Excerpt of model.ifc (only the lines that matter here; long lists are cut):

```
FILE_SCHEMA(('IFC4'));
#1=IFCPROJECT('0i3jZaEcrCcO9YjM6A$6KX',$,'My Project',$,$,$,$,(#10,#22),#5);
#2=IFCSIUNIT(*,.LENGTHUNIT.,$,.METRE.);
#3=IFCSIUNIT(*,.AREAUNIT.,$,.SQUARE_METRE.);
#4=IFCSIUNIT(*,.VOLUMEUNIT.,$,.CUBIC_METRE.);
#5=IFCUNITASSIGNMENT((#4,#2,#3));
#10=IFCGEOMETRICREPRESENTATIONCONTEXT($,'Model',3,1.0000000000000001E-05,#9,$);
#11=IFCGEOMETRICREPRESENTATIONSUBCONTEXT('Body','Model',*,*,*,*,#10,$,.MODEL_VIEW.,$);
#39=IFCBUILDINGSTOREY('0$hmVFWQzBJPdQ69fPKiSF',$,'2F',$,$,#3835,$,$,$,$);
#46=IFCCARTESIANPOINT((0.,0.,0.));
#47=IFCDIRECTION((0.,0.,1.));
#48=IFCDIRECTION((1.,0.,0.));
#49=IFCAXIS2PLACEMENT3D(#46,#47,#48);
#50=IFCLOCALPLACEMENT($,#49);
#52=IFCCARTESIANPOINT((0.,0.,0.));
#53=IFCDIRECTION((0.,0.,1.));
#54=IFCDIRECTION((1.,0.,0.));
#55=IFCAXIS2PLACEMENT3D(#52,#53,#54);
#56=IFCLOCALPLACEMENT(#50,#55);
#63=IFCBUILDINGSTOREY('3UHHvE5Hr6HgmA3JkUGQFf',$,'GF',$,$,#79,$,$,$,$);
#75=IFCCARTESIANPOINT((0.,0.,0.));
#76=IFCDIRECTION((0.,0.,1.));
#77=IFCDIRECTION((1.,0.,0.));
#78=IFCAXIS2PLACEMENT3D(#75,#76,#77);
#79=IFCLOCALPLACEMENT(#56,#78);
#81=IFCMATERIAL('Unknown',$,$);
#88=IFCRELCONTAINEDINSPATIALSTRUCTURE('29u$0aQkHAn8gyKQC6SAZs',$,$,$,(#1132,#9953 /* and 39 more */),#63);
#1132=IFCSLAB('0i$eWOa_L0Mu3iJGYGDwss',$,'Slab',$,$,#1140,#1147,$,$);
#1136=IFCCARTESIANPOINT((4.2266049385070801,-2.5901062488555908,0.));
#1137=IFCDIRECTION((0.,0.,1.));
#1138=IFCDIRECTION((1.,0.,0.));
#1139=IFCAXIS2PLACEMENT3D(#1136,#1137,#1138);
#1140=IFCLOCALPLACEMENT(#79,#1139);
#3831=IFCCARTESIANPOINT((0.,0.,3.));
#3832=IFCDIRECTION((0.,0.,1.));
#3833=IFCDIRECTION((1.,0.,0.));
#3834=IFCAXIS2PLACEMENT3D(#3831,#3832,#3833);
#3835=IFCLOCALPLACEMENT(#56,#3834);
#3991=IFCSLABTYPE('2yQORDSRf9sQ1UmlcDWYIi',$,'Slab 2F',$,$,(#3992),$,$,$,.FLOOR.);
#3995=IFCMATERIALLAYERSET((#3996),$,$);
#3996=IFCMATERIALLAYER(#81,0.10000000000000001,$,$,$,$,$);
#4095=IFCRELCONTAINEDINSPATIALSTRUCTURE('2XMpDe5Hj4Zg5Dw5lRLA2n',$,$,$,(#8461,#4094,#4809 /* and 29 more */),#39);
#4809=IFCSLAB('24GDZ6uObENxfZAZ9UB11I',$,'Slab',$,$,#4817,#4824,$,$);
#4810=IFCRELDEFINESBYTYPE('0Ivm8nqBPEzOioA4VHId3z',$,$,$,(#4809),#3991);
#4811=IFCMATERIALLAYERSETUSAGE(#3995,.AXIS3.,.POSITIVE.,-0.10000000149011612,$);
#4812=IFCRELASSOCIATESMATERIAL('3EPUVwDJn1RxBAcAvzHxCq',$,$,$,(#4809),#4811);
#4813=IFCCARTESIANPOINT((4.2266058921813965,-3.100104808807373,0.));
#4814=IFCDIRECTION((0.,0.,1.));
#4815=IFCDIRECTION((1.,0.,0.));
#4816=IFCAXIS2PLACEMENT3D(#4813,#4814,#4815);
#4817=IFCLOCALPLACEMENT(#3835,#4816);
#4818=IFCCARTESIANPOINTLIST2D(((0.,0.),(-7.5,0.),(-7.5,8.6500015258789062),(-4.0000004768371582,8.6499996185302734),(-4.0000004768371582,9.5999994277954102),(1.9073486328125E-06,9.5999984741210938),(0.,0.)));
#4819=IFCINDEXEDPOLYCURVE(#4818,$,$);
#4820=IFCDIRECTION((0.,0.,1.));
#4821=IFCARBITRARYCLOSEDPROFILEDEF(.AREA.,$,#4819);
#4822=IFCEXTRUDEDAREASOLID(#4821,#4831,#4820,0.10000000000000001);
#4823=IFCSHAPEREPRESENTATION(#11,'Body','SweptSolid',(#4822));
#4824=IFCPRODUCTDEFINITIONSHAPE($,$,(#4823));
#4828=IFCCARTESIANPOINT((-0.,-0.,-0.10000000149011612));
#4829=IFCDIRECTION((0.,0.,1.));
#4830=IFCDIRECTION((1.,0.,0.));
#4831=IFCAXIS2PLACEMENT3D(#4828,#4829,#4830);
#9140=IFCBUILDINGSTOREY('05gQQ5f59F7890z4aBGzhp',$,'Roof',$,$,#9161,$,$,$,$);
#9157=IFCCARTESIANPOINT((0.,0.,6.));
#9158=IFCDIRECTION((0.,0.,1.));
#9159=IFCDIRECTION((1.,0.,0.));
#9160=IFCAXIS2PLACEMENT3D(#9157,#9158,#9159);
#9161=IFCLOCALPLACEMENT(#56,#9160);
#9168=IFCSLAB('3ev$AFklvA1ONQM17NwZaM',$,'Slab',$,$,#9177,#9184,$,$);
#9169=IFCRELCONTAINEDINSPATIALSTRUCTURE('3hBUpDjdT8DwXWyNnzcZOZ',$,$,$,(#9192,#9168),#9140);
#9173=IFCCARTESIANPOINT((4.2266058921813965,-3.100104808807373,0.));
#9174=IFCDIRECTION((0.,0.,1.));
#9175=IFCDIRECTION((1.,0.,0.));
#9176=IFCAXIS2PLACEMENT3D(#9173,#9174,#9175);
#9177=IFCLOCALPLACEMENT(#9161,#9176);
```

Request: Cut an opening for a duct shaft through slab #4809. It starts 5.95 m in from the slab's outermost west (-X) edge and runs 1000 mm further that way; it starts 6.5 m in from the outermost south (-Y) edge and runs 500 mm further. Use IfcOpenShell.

```python
import numpy as np
import ifcopenshell
import ifcopenshell.api.feature
import ifcopenshell.api.geometry
import ifcopenshell.api.root
import ifcopenshell.geom
import ifcopenshell.util.placement
import ifcopenshell.util.representation
import ifcopenshell.util.shape
import ifcopenshell.util.unit

model = ifcopenshell.open("model.ifc")
unit_scale = ifcopenshell.util.unit.calculate_unit_scale(model)
settings = ifcopenshell.geom.settings()


def volume(element):
    """Net volume in cubic metres, openings subtracted."""
    shape = ifcopenshell.geom.create_shape(settings, element)
    return ifcopenshell.util.shape.get_volume(shape.geometry)


slab = model.by_guid("24GDZ6uObENxfZAZ9UB11I")
before = volume(slab)

# Extent in the slab's own axes, in metres. The edges named are its -X and -Y sides.
slab_shape = ifcopenshell.geom.create_shape(settings, slab)
vertices = ifcopenshell.util.shape.get_vertices(slab_shape.geometry)
x_min, y_min, bottom = vertices.min(axis=0)
top = vertices[:, 2].max()

opening = ifcopenshell.api.root.create_entity(model, ifc_class="IfcOpeningElement", name="Duct shaft opening", predefined_type="OPENING")
context = ifcopenshell.util.representation.get_context(model, "Model", "Body", "MODEL_VIEW")
width, depth = 1, 0.5
outline = [(0.0, 0.0), (width, 0.0), (width, depth), (0.0, depth), (0.0, 0.0)]
# Overshoot both faces by 50 mm so the cut is clean.
shape = ifcopenshell.api.geometry.add_slab_representation(
    model, context=context, depth=top - bottom + 0.1, polyline=outline
)
ifcopenshell.api.geometry.assign_representation(model, product=opening, representation=shape)

matrix = ifcopenshell.util.placement.get_local_placement(slab.ObjectPlacement)
matrix[:, 3] = matrix @ np.append(np.array([x_min + 5.95, y_min + 6.5, bottom - 0.05]) / unit_scale, 1.0)
ifcopenshell.api.geometry.edit_object_placement(model, product=opening, matrix=matrix, is_si=False)
ifcopenshell.api.feature.add_feature(model, feature=opening, element=slab)

after = volume(slab)

print(f"slab volume {before:.3f} -> {after:.3f} m3")

model.write("model_v2.ifc")
```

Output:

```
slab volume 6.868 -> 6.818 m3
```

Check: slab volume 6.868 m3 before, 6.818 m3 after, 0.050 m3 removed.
